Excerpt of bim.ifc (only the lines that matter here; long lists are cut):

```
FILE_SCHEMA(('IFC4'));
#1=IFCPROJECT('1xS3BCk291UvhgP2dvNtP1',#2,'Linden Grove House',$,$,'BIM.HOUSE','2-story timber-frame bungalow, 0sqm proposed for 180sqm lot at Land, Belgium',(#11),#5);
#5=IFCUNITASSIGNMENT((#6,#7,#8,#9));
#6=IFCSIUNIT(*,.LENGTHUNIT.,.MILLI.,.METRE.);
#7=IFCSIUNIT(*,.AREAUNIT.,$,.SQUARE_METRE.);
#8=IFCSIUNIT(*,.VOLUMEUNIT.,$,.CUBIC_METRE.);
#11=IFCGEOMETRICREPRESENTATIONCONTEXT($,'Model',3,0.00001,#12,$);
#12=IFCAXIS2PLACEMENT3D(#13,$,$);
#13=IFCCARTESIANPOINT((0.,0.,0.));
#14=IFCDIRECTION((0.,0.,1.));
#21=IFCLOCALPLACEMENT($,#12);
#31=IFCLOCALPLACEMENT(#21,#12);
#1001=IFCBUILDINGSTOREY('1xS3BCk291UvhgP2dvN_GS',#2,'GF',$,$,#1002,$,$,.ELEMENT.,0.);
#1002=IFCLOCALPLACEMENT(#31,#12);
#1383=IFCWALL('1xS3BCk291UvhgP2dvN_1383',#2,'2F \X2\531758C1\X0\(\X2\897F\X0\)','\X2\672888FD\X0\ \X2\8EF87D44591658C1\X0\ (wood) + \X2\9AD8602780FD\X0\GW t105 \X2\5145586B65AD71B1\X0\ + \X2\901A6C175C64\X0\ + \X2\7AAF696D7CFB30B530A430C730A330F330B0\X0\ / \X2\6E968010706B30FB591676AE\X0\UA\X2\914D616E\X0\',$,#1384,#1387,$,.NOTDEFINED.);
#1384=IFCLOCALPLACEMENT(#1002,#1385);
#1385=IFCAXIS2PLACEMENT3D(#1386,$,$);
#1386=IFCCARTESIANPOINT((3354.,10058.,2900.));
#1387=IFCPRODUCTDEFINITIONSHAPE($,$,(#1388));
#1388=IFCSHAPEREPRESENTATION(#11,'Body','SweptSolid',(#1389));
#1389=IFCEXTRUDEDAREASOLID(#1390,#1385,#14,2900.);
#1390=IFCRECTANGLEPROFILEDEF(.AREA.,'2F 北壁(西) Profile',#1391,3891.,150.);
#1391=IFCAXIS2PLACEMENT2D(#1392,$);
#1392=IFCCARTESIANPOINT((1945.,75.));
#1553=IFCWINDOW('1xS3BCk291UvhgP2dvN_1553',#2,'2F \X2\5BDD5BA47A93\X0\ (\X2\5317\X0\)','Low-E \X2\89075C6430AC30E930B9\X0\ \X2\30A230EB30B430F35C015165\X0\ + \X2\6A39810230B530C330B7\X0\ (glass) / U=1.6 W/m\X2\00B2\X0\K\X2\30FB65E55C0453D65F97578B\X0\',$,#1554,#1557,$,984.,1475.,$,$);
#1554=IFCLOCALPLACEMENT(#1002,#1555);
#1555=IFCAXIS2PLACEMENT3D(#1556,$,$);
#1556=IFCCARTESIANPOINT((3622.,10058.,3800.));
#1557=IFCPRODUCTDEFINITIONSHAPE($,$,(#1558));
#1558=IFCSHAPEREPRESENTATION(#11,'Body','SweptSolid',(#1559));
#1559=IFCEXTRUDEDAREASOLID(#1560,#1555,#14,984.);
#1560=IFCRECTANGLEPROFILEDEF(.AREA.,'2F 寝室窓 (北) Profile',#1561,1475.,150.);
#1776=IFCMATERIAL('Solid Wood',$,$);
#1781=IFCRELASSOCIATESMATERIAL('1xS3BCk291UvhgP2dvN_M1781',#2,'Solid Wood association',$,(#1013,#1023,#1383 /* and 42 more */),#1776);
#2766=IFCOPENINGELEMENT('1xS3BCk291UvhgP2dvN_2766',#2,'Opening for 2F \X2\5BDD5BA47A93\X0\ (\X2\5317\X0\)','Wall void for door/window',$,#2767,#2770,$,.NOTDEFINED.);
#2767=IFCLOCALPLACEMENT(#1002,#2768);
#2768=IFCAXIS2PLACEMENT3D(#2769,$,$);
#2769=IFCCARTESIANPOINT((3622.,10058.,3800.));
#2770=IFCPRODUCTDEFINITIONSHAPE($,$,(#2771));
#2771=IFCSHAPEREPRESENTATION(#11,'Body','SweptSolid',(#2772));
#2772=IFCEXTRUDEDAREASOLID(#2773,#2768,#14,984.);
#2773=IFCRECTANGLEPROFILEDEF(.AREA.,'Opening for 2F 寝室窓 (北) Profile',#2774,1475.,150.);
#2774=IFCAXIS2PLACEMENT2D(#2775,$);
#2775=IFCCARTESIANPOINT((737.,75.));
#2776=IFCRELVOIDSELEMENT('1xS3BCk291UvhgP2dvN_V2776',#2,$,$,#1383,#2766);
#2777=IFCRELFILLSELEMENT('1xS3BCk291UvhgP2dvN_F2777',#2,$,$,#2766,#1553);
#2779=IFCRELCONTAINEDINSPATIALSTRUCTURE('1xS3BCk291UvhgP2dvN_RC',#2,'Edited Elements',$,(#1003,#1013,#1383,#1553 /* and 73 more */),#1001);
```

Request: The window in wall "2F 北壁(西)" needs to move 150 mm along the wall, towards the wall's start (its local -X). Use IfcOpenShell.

```python
import ifcopenshell
import ifcopenshell.api.geometry
import ifcopenshell.util.placement

model = ifcopenshell.open("bim.ifc")

window = model.by_id(1553)
opening = window.FillsVoids[0].RelatingOpeningElement
wall = opening.VoidsElements[0].RelatingBuildingElement

wall_matrix = ifcopenshell.util.placement.get_local_placement(wall.ObjectPlacement)
shift = wall_matrix[:3, 0] * -150.0
before = ifcopenshell.util.placement.get_local_placement(window.ObjectPlacement)[:3, 3].copy()

# The window is not placed relative to its opening, so move both.
for product in (opening, window):
    matrix = ifcopenshell.util.placement.get_local_placement(product.ObjectPlacement)
    matrix[:3, 3] += shift
    ifcopenshell.api.geometry.edit_object_placement(model, product=product, matrix=matrix, is_si=False)

after = ifcopenshell.util.placement.get_local_placement(window.ObjectPlacement)[:3, 3]
print("window moved by", (after - before).round(3) + 0.0)

model.write("bim_edited.ifc")
```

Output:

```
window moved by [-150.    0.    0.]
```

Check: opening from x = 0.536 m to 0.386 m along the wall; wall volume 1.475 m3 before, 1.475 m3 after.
